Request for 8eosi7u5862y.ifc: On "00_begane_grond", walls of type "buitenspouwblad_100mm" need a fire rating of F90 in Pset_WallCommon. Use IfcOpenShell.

First a look at what the model holds.

```python
import ifcopenshell
import ifcopenshell.util.element

model = ifcopenshell.open("8eosi7u5862y.ifc")
print(model.schema)
storey = next(s for s in model.by_type("IfcBuildingStorey") if s.Name == "00_begane_grond")
walls = [e for e in ifcopenshell.util.element.get_decomposition(storey) if e.is_a("IfcWall")]
seen = {}
for e in walls:
    element_type = ifcopenshell.util.element.get_type(e)
    key = (element_type.Name if element_type != e and element_type else None, ifcopenshell.util.element.get_pset(e, "Pset_WallCommon", "FireRating"))
    seen[key] = seen.get(key, 0) + 1
for (name, value), count in sorted(seen.items(), key=str):
    print(count, "x", name, "|", value)
```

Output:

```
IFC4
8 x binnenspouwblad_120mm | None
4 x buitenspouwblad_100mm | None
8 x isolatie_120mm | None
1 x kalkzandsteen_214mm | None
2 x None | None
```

```python
import ifcopenshell
import ifcopenshell.api.pset
import ifcopenshell.util.element

model = ifcopenshell.open("8eosi7u5862y.ifc")

storey = next(s for s in model.by_type("IfcBuildingStorey") if s.Name == "00_begane_grond")
walls = [e for e in ifcopenshell.util.element.get_decomposition(storey) if e.is_a("IfcWall")]

count = 0
for e in walls:
    element_type = ifcopenshell.util.element.get_type(e)
    if element_type in (None, e) or element_type.Name != "buitenspouwblad_100mm":
        continue
    # add_pset returns the element's existing set when there is one.
    pset = ifcopenshell.api.pset.add_pset(model, product=e, name="Pset_WallCommon")
    ifcopenshell.api.pset.edit_pset(model, pset=pset, properties={"FireRating": "F90"})
    count += 1

print(count, "walls updated")

model.write("8eosi7u5862y_edited.ifc")
```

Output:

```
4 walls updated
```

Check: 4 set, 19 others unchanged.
